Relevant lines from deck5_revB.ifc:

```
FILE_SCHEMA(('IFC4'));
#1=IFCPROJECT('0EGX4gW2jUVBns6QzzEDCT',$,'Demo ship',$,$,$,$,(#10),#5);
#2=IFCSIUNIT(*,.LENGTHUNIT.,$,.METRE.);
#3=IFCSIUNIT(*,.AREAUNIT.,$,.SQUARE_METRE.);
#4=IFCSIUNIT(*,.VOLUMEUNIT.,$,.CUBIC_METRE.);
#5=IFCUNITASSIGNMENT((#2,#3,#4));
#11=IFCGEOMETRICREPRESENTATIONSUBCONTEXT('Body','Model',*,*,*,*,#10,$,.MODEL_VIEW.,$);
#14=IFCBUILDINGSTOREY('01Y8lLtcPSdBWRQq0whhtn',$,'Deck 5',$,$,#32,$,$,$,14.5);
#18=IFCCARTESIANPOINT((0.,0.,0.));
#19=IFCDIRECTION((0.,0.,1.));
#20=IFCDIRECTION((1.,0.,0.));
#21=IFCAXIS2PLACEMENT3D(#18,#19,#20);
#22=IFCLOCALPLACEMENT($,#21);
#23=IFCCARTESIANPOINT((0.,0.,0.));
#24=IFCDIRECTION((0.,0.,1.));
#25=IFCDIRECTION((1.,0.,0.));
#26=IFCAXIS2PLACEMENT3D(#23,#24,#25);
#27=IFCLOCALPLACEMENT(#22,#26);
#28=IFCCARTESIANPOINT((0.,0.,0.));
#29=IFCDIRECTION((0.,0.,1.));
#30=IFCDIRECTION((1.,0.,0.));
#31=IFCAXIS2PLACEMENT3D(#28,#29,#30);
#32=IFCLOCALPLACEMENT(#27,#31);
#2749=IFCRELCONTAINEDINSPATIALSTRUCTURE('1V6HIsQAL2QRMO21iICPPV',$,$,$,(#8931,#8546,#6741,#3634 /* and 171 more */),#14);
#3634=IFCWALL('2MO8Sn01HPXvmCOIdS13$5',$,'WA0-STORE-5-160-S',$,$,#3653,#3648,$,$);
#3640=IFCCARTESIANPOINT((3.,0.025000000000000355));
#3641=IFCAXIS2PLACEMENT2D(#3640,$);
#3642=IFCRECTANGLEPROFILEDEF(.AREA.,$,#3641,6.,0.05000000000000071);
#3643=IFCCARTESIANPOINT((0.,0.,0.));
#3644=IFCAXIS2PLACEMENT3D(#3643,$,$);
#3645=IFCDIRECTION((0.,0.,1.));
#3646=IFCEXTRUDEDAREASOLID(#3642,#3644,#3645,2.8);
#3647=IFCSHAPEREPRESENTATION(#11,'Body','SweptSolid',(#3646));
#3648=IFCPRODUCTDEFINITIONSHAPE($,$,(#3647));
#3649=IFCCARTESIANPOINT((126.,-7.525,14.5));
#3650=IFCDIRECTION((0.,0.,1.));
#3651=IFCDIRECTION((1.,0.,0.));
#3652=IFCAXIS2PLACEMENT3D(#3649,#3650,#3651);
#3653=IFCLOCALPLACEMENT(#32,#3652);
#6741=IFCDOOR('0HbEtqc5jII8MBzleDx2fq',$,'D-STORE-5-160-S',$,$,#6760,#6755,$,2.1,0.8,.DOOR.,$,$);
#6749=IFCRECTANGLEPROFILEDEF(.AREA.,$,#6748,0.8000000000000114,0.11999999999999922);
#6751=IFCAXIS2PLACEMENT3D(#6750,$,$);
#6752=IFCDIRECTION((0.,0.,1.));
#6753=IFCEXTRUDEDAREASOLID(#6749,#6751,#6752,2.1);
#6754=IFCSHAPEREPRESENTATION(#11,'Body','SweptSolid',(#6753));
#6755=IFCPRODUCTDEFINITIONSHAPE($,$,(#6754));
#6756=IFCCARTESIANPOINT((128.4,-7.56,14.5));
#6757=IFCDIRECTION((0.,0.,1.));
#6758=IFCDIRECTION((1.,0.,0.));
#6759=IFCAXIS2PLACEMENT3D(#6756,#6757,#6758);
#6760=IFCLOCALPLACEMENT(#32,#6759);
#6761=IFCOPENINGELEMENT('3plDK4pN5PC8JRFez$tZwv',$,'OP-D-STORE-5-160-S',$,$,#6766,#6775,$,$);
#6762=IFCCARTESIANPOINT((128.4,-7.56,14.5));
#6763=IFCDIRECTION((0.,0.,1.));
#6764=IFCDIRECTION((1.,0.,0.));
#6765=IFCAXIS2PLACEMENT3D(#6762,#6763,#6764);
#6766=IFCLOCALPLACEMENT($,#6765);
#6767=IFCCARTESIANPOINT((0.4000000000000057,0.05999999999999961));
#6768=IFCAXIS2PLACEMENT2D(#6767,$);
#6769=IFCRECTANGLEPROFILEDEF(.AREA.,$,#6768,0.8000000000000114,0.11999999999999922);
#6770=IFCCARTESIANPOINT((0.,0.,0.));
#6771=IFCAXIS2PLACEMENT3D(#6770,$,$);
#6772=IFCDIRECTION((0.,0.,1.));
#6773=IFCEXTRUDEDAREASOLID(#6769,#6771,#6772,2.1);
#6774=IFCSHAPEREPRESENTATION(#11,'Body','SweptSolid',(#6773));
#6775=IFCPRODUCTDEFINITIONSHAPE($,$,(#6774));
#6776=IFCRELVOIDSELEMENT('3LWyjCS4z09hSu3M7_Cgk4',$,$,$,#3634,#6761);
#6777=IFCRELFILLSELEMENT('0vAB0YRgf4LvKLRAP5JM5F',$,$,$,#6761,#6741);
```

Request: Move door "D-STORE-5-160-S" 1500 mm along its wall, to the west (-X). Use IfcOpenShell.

```python
import ifcopenshell
import ifcopenshell.api.geometry
import ifcopenshell.util.placement

model = ifcopenshell.open("deck5_revB.ifc")

door = model.by_guid("0HbEtqc5jII8MBzleDx2fq")
opening = door.FillsVoids[0].RelatingOpeningElement
wall = opening.VoidsElements[0].RelatingBuildingElement

wall_matrix = ifcopenshell.util.placement.get_local_placement(wall.ObjectPlacement)
shift = wall_matrix[:3, 0] * -1.5
before = ifcopenshell.util.placement.get_local_placement(door.ObjectPlacement)[:3, 3].copy()

# The door is not placed relative to its opening, so move both.
for product in (opening, door):
    matrix = ifcopenshell.util.placement.get_local_placement(product.ObjectPlacement)
    matrix[:3, 3] += shift
    ifcopenshell.api.geometry.edit_object_placement(model, product=product, matrix=matrix, is_si=False)

after = ifcopenshell.util.placement.get_local_placement(door.ObjectPlacement)[:3, 3]
print("door moved by", (after - before).round(3) + 0.0)

model.write("deck5_revB_edited.ifc")
```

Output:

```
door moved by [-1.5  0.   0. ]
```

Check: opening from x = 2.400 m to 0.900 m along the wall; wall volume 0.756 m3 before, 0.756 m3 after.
